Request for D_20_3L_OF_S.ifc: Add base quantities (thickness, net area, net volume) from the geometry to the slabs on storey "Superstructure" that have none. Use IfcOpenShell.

First a look at what the model holds.

```python
import ifcopenshell
import ifcopenshell.util.element
import ifcopenshell.util.unit

model = ifcopenshell.open("D_20_3L_OF_S.ifc")
print(model.schema)
for unit_type in ("LENGTHUNIT", "AREAUNIT", "VOLUMEUNIT"):
    print(unit_type, ifcopenshell.util.unit.calculate_unit_scale(model, unit_type))
storey = next(s for s in model.by_type("IfcBuildingStorey") if s.Name == "Superstructure")
slabs = [e for e in ifcopenshell.util.element.get_decomposition(storey) if e.is_a("IfcSlab")]
for e in sorted(slabs, key=lambda e: e.id()):
    print(e.id(), e.is_a(), e.Name, list(ifcopenshell.util.element.get_psets(e, qtos_only=True)), sep=" | ")
```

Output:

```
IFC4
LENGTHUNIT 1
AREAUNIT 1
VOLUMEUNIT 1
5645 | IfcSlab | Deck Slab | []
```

```python
import ifcopenshell
import ifcopenshell.api.pset
import ifcopenshell.geom
import ifcopenshell.util.element
import ifcopenshell.util.shape
import ifcopenshell.util.unit

model = ifcopenshell.open("D_20_3L_OF_S.ifc")
unit_scale = ifcopenshell.util.unit.calculate_unit_scale(model)
area_scale = ifcopenshell.util.unit.calculate_unit_scale(model, "AREAUNIT")
volume_scale = ifcopenshell.util.unit.calculate_unit_scale(model, "VOLUMEUNIT")
settings = ifcopenshell.geom.settings()

storey = next(s for s in model.by_type("IfcBuildingStorey") if s.Name == "Superstructure")
slabs = [e for e in ifcopenshell.util.element.get_decomposition(storey) if e.is_a("IfcSlab")]

for e in sorted(slabs, key=lambda e: e.id()):
    if ifcopenshell.util.element.get_psets(e, qtos_only=True, should_inherit=False):
        continue
    # Geometry comes back in metres, in the element's own axes.
    shape = ifcopenshell.geom.create_shape(settings, e)
    values = {
        "Width": ifcopenshell.util.shape.get_z(shape.geometry) / unit_scale,
        "NetArea": ifcopenshell.util.shape.get_footprint_area(shape.geometry) / area_scale,
        "NetVolume": ifcopenshell.util.shape.get_volume(shape.geometry) / volume_scale,
    }
    qto = ifcopenshell.api.pset.add_qto(model, product=e, name="Qto_SlabBaseQuantities")
    ifcopenshell.api.pset.edit_qto(model, qto=qto, properties=values)
    print(e.id(), {k: round(v, 3) for k, v in values.items()})

model.write("D_20_3L_OF_S_rev.ifc")
```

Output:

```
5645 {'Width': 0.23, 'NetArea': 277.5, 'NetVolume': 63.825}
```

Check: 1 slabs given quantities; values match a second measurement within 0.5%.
